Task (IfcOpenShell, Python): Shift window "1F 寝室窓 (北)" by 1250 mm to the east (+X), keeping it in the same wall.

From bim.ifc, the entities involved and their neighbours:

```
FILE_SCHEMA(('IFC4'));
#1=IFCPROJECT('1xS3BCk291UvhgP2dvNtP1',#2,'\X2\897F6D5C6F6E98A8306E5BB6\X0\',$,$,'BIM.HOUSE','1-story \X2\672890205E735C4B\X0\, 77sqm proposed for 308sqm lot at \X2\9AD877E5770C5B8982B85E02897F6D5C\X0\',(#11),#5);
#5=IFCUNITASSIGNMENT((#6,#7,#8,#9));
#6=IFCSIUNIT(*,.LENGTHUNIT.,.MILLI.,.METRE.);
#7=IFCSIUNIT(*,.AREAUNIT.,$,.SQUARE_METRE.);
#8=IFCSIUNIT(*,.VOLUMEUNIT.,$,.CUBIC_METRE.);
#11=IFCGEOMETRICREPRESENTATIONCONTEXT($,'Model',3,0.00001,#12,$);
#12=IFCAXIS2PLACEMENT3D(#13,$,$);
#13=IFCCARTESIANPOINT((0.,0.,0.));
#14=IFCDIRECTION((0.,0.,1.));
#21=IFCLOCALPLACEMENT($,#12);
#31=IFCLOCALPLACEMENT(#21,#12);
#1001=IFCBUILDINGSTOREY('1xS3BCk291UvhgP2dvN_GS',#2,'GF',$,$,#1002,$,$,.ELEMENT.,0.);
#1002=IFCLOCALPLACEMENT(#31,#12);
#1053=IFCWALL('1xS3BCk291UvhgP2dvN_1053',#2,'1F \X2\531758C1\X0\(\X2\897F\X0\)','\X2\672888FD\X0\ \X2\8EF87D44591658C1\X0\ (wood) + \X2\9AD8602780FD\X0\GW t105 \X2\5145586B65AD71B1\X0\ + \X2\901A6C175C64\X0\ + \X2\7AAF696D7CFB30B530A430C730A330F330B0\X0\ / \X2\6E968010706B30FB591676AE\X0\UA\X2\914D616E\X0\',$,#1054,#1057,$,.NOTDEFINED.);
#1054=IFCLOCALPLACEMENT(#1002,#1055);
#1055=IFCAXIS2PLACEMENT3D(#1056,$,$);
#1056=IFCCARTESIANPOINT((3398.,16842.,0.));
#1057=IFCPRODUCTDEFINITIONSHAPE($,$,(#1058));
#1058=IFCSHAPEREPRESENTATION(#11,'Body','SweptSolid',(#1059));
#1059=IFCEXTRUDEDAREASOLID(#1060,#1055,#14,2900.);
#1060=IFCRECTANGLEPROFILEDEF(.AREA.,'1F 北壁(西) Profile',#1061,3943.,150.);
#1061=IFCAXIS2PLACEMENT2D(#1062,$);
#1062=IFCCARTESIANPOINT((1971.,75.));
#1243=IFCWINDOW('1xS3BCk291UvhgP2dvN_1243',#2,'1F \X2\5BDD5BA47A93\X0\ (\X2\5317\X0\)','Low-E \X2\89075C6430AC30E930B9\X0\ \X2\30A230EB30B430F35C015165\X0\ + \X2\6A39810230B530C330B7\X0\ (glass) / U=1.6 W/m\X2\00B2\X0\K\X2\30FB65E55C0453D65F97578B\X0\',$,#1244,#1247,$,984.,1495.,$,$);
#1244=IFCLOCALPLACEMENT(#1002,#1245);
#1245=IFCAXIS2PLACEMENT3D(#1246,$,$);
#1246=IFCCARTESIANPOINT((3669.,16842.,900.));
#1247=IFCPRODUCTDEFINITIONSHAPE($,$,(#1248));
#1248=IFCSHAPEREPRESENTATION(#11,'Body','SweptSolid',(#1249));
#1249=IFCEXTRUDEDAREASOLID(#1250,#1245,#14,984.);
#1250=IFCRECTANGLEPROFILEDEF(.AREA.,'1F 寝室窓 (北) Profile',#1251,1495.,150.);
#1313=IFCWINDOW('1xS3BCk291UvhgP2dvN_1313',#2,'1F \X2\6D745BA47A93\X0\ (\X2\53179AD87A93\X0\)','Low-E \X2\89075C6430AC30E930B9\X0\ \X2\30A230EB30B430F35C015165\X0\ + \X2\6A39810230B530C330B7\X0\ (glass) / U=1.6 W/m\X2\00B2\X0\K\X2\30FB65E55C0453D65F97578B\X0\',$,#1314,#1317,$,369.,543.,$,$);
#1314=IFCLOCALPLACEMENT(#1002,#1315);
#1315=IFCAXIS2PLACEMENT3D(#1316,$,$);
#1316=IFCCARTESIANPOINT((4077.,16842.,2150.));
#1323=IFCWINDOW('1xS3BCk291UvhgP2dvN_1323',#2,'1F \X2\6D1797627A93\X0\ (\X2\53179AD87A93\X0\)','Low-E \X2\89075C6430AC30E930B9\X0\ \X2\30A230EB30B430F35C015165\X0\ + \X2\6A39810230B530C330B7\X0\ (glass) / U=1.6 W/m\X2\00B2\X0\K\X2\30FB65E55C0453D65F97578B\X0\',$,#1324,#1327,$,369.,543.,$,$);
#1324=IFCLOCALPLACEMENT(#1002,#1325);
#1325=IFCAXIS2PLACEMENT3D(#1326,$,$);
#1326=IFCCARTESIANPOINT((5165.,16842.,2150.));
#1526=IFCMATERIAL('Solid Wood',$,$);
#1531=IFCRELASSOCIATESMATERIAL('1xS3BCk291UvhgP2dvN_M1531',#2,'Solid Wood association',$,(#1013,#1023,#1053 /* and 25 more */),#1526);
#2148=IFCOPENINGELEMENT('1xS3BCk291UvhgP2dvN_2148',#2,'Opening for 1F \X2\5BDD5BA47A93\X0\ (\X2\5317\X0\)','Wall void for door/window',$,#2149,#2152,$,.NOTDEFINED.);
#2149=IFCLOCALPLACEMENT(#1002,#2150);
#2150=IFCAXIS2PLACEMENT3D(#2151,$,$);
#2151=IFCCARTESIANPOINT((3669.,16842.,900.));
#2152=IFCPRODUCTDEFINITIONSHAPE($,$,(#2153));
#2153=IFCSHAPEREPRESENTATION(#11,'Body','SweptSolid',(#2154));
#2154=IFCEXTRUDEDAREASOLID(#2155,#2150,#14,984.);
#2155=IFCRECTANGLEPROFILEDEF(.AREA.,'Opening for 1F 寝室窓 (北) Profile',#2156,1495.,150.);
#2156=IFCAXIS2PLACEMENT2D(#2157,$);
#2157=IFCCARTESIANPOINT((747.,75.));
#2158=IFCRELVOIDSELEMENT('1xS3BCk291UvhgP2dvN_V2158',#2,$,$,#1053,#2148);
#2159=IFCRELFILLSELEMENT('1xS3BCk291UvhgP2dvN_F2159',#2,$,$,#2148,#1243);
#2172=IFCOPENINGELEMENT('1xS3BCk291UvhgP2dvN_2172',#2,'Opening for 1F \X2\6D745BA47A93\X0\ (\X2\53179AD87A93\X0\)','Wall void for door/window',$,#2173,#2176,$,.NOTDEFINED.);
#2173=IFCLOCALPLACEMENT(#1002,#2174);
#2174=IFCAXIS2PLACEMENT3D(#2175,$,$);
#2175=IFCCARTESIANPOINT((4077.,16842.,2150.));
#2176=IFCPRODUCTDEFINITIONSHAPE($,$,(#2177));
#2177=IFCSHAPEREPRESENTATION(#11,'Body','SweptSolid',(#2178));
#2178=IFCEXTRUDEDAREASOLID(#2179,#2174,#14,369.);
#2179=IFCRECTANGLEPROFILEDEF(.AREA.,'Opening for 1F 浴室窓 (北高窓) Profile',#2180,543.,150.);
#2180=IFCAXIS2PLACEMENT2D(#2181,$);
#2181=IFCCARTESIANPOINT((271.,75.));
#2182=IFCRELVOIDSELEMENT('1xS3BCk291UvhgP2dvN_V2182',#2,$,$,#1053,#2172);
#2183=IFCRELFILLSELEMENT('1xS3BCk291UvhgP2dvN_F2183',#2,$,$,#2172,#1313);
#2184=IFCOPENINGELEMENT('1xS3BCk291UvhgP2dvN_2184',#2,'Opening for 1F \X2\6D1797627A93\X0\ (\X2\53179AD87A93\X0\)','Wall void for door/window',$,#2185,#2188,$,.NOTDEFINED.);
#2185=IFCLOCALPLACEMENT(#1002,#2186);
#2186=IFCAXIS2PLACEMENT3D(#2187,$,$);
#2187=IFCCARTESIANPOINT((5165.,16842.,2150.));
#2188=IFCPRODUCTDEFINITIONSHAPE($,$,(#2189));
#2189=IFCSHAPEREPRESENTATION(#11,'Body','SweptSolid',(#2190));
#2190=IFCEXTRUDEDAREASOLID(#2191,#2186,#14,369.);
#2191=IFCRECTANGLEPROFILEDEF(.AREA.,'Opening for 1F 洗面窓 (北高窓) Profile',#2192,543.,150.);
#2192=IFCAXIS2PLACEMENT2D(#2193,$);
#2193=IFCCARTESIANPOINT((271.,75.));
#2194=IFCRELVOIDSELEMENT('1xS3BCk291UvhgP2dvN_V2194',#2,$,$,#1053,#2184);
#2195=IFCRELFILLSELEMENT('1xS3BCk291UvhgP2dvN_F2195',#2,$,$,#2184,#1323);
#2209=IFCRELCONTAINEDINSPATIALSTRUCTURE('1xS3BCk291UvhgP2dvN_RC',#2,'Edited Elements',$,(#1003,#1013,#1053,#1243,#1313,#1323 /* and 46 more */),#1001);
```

```python
import ifcopenshell
import ifcopenshell.api.geometry
import ifcopenshell.util.placement
import ifcopenshell.util.unit

model = ifcopenshell.open("bim.ifc")
unit_scale = ifcopenshell.util.unit.calculate_unit_scale(model)

window = model.by_guid("1xS3BCk291UvhgP2dvN_1243")
opening = window.FillsVoids[0].RelatingOpeningElement
wall = opening.VoidsElements[0].RelatingBuildingElement

wall_matrix = ifcopenshell.util.placement.get_local_placement(wall.ObjectPlacement)
shift = wall_matrix[:3, 0] * 1.25 / unit_scale
before = ifcopenshell.util.placement.get_local_placement(window.ObjectPlacement)[:3, 3].copy()

# The window is not placed relative to its opening, so move both.
for product in (opening, window):
    matrix = ifcopenshell.util.placement.get_local_placement(product.ObjectPlacement)
    matrix[:3, 3] += shift
    ifcopenshell.api.geometry.edit_object_placement(model, product=product, matrix=matrix, is_si=False)

after = ifcopenshell.util.placement.get_local_placement(window.ObjectPlacement)[:3, 3]
print("window moved by", (after - before).round(3) + 0.0)

model.write("bim_v2.ifc")
```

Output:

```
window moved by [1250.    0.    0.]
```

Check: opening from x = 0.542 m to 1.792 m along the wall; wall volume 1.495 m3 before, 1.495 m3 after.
